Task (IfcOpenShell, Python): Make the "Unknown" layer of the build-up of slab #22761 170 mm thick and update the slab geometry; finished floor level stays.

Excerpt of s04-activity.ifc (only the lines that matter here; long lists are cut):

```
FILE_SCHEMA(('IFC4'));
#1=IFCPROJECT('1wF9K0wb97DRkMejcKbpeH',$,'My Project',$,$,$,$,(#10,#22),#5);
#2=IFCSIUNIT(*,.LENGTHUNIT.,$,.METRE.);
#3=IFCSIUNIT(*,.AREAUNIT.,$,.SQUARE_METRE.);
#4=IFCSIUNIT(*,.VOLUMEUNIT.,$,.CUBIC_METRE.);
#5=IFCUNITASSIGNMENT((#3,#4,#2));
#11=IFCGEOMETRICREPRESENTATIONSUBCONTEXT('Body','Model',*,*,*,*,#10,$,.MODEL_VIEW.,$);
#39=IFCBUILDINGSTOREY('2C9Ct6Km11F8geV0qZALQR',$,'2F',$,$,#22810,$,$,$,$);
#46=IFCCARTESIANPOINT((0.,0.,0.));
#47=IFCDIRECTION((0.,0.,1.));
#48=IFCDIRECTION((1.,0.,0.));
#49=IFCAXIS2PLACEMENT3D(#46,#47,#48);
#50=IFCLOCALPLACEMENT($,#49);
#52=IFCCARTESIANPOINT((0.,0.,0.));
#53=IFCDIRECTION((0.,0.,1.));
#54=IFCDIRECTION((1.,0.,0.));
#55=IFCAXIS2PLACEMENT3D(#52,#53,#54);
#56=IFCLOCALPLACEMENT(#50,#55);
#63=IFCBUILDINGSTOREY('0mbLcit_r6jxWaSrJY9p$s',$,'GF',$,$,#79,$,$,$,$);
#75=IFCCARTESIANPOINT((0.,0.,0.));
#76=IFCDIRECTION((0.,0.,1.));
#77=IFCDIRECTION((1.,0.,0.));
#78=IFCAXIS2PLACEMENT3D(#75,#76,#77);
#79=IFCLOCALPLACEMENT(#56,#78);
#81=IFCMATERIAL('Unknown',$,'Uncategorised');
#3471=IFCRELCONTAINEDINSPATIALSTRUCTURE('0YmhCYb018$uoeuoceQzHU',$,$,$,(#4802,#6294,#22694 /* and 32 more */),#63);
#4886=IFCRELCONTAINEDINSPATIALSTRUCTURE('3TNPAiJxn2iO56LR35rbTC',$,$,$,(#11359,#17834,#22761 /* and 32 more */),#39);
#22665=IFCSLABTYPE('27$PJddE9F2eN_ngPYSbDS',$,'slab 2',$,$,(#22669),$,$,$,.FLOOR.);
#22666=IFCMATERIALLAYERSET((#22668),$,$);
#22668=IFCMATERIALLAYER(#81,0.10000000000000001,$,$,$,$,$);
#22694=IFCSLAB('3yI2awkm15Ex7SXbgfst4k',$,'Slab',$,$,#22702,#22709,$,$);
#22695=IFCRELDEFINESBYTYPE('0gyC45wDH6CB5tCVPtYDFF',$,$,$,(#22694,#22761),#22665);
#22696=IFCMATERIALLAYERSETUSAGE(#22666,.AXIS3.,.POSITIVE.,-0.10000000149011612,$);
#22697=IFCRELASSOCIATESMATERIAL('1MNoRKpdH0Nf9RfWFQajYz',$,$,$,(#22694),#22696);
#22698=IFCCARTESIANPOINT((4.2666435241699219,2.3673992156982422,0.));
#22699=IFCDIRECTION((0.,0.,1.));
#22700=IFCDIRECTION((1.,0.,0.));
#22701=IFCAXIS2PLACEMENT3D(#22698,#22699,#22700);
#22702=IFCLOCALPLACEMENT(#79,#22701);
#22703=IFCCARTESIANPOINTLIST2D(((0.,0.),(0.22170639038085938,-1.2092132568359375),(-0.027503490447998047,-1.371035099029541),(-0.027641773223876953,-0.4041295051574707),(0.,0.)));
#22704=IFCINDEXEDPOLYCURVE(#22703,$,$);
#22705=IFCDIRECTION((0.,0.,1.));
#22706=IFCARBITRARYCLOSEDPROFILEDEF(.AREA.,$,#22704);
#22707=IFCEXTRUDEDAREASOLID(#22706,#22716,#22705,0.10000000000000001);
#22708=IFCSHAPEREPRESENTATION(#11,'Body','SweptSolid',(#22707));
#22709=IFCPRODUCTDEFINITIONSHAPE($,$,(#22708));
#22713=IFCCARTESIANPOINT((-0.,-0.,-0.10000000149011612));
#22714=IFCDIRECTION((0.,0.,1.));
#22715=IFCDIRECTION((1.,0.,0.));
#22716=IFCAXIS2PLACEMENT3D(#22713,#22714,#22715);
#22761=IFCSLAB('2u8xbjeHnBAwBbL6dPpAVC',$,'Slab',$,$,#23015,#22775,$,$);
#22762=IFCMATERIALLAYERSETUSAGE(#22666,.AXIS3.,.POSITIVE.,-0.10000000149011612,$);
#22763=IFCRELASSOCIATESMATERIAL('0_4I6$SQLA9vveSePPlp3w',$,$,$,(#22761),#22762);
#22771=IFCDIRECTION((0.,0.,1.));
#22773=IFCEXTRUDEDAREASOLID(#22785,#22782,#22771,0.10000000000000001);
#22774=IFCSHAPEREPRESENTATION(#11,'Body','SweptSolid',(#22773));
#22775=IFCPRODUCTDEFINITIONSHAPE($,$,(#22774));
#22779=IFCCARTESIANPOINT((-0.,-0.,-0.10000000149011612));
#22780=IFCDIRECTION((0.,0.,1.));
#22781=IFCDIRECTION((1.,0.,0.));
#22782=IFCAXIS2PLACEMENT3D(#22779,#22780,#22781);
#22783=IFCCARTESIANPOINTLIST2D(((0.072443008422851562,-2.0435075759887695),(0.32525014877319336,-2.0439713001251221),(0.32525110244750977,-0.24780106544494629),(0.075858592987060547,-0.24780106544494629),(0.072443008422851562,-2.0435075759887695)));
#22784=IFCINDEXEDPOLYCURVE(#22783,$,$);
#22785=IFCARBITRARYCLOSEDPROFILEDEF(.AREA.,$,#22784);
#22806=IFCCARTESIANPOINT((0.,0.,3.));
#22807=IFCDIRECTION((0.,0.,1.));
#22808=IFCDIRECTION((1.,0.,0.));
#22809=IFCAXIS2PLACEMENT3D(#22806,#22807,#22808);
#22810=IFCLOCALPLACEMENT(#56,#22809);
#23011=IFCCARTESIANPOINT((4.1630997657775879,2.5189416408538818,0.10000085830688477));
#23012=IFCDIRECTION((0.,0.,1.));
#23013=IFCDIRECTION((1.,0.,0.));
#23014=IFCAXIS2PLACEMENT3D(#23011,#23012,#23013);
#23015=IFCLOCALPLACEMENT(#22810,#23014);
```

```python
import ifcopenshell
import ifcopenshell.util.element
import ifcopenshell.util.representation
import ifcopenshell.util.unit

model = ifcopenshell.open("s04-activity.ifc")
unit_scale = ifcopenshell.util.unit.calculate_unit_scale(model)

layer_set = model.by_id(22666)
layer = next(l for l in layer_set.MaterialLayers if l.Material and l.Material.Name == "Unknown")
change = 0.17 / unit_scale - layer.LayerThickness
layer.LayerThickness += change

# The layer set is shared, so every slab that uses it gets the new thickness.
slabs = [e for e in ifcopenshell.util.element.get_elements_by_material(model, layer_set) if e.is_a("IfcSlab")]
for slab in sorted(slabs, key=lambda e: e.id()):
    body = ifcopenshell.util.representation.get_representation(slab, "Model", "Body")
    solid = body.Items[0]
    old_depth = solid.Depth
    solid.Depth += change
    # Extruded upwards: lower the start of the extrusion so the top stays.
    x, y, z = solid.Position.Location.Coordinates
    solid.Position.Location = model.createIfcCartesianPoint((x, y, z - change))
    print(slab.id(), f"{old_depth:g} -> {solid.Depth:g}")

# The layers are counted up from the underside, which has moved.
for usage in {ifcopenshell.util.element.get_material(slab) for slab in slabs}:
    usage.OffsetFromReferenceLine -= change

model.write("s04-activity_edited.ifc")
```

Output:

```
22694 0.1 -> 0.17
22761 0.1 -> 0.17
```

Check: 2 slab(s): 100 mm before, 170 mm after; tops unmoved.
